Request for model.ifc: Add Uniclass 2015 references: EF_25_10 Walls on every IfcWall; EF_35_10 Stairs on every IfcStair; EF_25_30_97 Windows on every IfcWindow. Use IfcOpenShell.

First a look at what the model holds.

```python
import ifcopenshell

model = ifcopenshell.open("model.ifc")
print(model.schema)
print("classifications:", [c.Name for c in model.by_type("IfcClassification")])
for ifc_class in ("IfcDoor", "IfcRoof", "IfcStair", "IfcWall", "IfcWindow"):
    print(ifc_class, len(model.by_type(ifc_class)))
```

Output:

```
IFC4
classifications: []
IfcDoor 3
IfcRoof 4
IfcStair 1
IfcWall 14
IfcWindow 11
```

```python
import ifcopenshell
import ifcopenshell.api.classification

model = ifcopenshell.open("model.ifc")

system = ifcopenshell.api.classification.add_classification(model, classification="Uniclass 2015")

codes = {
    "IfcWall": ("EF_25_10", "Walls"),
    "IfcStair": ("EF_35_10", "Stairs"),
    "IfcWindow": ("EF_25_30_97", "Windows"),
}
for ifc_class, (code, name) in codes.items():
    products = model.by_type(ifc_class)
    ifcopenshell.api.classification.add_reference(
        model, products=products, classification=system, identification=code, name=name
    )
    print(code, len(products))

model.write("model_updated.ifc")
```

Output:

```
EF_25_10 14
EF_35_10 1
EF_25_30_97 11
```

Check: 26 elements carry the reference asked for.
